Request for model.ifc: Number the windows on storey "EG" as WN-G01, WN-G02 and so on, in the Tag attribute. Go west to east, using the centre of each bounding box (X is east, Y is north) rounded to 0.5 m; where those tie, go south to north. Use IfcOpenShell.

First a look at what the model holds.

```python
import ifcopenshell
import ifcopenshell.util.element
import ifcopenshell.util.placement

model = ifcopenshell.open("model.ifc")
print(model.schema)
storey = next(s for s in model.by_type("IfcBuildingStorey") if s.Name == "EG")
windows = [e for e in ifcopenshell.util.element.get_decomposition(storey) if e.is_a("IfcWindow")]
for e in sorted(windows, key=lambda e: e.id()):
    origin = ifcopenshell.util.placement.get_local_placement(e.ObjectPlacement)[:3, 3]
    print(e.id(), e.Tag, e.Name, origin.round(2) + 0.0, sep=" | ")
```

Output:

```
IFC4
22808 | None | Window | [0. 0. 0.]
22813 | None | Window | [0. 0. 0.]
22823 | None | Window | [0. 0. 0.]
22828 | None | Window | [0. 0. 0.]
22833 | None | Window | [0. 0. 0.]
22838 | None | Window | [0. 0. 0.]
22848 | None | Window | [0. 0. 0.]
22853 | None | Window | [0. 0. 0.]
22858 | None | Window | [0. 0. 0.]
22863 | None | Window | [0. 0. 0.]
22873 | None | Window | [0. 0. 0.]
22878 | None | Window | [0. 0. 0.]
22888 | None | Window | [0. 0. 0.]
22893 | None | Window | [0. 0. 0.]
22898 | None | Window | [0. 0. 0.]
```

```python
import ifcopenshell
import ifcopenshell.geom
import ifcopenshell.util.element
import ifcopenshell.util.shape

model = ifcopenshell.open("model.ifc")
settings = ifcopenshell.geom.settings()
settings.set("use-world-coords", True)


def centre(element):
    shape = ifcopenshell.geom.create_shape(settings, element)
    return ifcopenshell.util.shape.get_bbox_centroid(shape.geometry)


storey = next(s for s in model.by_type("IfcBuildingStorey") if s.Name == "EG")
windows = [e for e in ifcopenshell.util.element.get_decomposition(storey) if e.is_a("IfcWindow")]

# Insertion points can sit at a corner or the storey origin, so sort by the geometry (in metres).
centres = {e: centre(e) for e in windows}
windows.sort(key=lambda e: (round(centres[e][0] / 0.5), centres[e][1]))

for i, e in enumerate(windows, start=1):
    number = f"WN-G{i:02d}"
    e.Tag = number
    print(e.id(), number)

model.write("model_updated.ifc")
```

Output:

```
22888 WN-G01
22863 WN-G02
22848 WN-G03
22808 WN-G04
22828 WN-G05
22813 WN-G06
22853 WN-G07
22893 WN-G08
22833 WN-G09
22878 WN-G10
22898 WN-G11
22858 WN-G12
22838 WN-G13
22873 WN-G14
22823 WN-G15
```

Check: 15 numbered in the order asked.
